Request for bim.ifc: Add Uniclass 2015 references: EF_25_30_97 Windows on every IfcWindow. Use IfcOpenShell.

First a look at what the model holds.

```python
import ifcopenshell

model = ifcopenshell.open("bim.ifc")
print(model.schema)
print("classifications:", [c.Name for c in model.by_type("IfcClassification")])
for ifc_class in ("IfcDoor", "IfcRoof", "IfcStair", "IfcWall", "IfcWindow"):
    print(ifc_class, len(model.by_type(ifc_class)))
```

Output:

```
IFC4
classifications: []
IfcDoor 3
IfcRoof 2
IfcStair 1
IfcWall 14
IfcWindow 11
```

```python
import ifcopenshell
import ifcopenshell.api.classification

model = ifcopenshell.open("bim.ifc")

system = ifcopenshell.api.classification.add_classification(model, classification="Uniclass 2015")

codes = {
    "IfcWindow": ("EF_25_30_97", "Windows"),
}
for ifc_class, (code, name) in codes.items():
    products = model.by_type(ifc_class)
    ifcopenshell.api.classification.add_reference(
        model, products=products, classification=system, identification=code, name=name
    )
    print(code, len(products))

model.write("bim_rev.ifc")
```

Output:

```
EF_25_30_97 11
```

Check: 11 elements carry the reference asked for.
